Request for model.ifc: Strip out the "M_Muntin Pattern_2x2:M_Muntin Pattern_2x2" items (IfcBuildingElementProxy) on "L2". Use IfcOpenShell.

First a look at what the model holds.

```python
import ifcopenshell
import ifcopenshell.util.element

model = ifcopenshell.open("model.ifc")
print(model.schema)
storey = next(s for s in model.by_type("IfcBuildingStorey") if s.Name == "L2")
proxies = [e for e in ifcopenshell.util.element.get_decomposition(storey) if e.is_a("IfcBuildingElementProxy")]
seen = {}
for e in proxies:
    element_type = ifcopenshell.util.element.get_type(e)
    name = element_type.Name if element_type not in (None, e) else None
    seen[name] = seen.get(name, 0) + 1
for name, count in sorted(seen.items(), key=str):
    print(count, "x", name)
```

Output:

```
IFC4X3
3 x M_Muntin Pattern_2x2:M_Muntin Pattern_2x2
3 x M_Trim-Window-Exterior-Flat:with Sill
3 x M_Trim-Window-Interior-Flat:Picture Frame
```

```python
import ifcopenshell
import ifcopenshell.api.root
import ifcopenshell.util.element

model = ifcopenshell.open("model.ifc")

storey = next(s for s in model.by_type("IfcBuildingStorey") if s.Name == "L2")
proxies = [e for e in ifcopenshell.util.element.get_decomposition(storey) if e.is_a("IfcBuildingElementProxy")]
targets = [e for e in proxies if (t := ifcopenshell.util.element.get_type(e)) not in (None, e) and t.Name == "M_Muntin Pattern_2x2:M_Muntin Pattern_2x2"]

for e in targets:
    ifcopenshell.api.root.remove_product(model, product=e)
print(len(targets), "removed")

model.write("model_rev.ifc")
```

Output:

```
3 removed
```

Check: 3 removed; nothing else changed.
